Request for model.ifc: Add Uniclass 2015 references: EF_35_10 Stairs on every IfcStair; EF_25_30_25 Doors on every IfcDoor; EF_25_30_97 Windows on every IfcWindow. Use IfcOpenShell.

First a look at what the model holds.

```python
import ifcopenshell

model = ifcopenshell.open("model.ifc")
print(model.schema)
print("classifications:", [c.Name for c in model.by_type("IfcClassification")])
for ifc_class in ("IfcDoor", "IfcRoof", "IfcStair", "IfcWall", "IfcWindow"):
    print(ifc_class, len(model.by_type(ifc_class)))
```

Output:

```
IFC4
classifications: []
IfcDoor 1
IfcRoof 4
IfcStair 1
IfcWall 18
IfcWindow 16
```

```python
import ifcopenshell
import ifcopenshell.api.classification

model = ifcopenshell.open("model.ifc")

system = ifcopenshell.api.classification.add_classification(model, classification="Uniclass 2015")

codes = {
    "IfcStair": ("EF_35_10", "Stairs"),
    "IfcDoor": ("EF_25_30_25", "Doors"),
    "IfcWindow": ("EF_25_30_97", "Windows"),
}
for ifc_class, (code, name) in codes.items():
    products = model.by_type(ifc_class)
    ifcopenshell.api.classification.add_reference(
        model, products=products, classification=system, identification=code, name=name
    )
    print(code, len(products))

model.write("model_updated.ifc")
```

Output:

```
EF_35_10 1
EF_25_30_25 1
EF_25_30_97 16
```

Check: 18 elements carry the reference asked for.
